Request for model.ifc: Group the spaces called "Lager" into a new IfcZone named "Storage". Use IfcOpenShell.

First a look at what the model holds.

```python
import ifcopenshell

model = ifcopenshell.open("model.ifc")
print(model.schema)
seen = {}
for space in model.by_type("IfcSpace"):
    seen[space.LongName] = seen.get(space.LongName, 0) + 1
for name, count in sorted(seen.items(), key=str):
    print(count, "x", name)
print("zones:", [z.Name for z in model.by_type("IfcZone")][:20])
```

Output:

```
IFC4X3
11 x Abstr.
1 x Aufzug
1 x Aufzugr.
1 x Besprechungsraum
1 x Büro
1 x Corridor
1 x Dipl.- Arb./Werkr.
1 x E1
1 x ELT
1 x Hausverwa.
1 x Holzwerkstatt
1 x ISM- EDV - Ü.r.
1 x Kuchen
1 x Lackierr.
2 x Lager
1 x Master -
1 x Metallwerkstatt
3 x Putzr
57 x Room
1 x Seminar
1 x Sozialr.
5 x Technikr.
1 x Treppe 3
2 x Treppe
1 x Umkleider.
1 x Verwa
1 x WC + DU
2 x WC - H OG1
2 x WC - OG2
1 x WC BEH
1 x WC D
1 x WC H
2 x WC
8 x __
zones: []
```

```python
import ifcopenshell
import ifcopenshell.api.group
import ifcopenshell.api.root

model = ifcopenshell.open("model.ifc")

names = {"Lager"}
spaces = [s for s in model.by_type("IfcSpace") if s.LongName in names]

zone = ifcopenshell.api.root.create_entity(model, ifc_class="IfcZone", name="Storage")
ifcopenshell.api.group.assign_group(model, products=spaces, group=zone)
print(len(spaces), "spaces in", zone.Name)

model.write("model_edited.ifc")
```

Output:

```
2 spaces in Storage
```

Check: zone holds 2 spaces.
